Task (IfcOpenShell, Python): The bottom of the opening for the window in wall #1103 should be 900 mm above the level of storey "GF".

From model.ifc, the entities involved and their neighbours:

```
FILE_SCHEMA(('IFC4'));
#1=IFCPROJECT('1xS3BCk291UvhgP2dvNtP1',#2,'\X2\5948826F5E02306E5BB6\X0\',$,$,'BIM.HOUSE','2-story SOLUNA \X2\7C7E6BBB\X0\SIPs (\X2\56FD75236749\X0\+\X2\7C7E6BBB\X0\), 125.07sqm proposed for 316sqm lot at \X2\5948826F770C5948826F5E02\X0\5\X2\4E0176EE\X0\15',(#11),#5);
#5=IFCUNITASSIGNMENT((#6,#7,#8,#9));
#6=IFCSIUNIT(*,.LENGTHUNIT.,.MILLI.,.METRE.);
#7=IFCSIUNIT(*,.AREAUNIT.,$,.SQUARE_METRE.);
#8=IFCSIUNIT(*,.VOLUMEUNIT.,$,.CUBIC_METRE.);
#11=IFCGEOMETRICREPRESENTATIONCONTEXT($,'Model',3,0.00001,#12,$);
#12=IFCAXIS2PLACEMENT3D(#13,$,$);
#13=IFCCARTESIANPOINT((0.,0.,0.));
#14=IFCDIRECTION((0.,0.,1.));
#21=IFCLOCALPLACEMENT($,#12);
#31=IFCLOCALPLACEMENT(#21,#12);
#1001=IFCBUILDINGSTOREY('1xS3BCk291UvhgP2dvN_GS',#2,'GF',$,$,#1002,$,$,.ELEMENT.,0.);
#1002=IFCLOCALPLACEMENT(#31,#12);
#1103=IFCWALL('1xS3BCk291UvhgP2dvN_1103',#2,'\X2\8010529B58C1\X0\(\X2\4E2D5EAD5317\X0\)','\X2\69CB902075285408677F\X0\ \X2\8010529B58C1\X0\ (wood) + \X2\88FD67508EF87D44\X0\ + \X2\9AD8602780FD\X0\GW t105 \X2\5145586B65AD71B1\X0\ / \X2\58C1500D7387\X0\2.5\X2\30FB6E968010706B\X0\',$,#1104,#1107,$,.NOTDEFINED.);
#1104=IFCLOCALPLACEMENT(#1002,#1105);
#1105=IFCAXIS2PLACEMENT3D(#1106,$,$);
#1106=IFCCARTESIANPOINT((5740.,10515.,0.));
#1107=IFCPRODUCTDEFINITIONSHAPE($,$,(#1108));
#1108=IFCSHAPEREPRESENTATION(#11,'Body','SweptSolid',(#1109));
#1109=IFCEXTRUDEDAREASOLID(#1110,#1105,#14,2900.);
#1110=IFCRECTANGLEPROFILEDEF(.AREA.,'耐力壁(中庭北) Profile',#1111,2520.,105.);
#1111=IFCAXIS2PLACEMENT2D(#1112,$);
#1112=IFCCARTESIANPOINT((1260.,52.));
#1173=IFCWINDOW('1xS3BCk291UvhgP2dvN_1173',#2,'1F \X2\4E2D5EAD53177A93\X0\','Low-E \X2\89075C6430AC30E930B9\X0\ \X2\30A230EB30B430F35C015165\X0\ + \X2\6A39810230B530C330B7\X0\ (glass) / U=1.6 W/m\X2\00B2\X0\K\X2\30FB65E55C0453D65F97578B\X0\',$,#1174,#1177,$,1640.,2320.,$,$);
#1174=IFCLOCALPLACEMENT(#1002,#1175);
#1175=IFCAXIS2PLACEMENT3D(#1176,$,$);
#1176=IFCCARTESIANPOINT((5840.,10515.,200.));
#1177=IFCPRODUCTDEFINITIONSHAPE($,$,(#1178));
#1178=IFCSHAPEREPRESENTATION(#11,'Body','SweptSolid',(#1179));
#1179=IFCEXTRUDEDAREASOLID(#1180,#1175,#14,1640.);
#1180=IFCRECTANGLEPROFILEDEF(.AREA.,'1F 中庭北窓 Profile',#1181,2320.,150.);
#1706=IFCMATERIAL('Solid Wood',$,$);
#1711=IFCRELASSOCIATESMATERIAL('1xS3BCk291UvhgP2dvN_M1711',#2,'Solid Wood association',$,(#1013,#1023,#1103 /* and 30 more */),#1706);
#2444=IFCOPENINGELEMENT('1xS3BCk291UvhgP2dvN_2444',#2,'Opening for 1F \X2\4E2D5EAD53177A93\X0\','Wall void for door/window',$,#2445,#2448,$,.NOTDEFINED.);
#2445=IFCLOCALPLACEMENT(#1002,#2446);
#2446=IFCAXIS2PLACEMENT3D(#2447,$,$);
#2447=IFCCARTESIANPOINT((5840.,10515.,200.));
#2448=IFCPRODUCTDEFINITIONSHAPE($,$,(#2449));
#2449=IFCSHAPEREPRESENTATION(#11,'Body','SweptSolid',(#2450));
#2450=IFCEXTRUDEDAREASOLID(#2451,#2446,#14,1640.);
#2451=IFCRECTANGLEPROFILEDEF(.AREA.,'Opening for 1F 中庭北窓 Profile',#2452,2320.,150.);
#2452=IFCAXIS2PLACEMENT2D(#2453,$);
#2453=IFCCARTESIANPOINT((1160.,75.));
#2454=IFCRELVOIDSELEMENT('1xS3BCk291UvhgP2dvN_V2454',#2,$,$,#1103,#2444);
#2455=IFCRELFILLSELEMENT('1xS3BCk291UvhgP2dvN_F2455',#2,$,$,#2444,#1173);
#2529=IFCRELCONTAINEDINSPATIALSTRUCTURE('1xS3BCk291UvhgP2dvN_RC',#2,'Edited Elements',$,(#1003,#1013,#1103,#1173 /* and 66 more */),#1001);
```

```python
import numpy as np
import ifcopenshell
import ifcopenshell.api.geometry
import ifcopenshell.geom
import ifcopenshell.util.element
import ifcopenshell.util.placement
import ifcopenshell.util.shape
import ifcopenshell.util.unit

model = ifcopenshell.open("model.ifc")
unit_scale = ifcopenshell.util.unit.calculate_unit_scale(model)

window = model.by_guid("1xS3BCk291UvhgP2dvN_1173")
opening = window.FillsVoids[0].RelatingOpeningElement
storey = ifcopenshell.util.element.get_container(window, ifc_class="IfcBuildingStorey")
level = ifcopenshell.util.placement.get_local_placement(storey.ObjectPlacement)[2, 3]

# The opening's origin need not be at the sill, so measure its lowest point.
shape = ifcopenshell.geom.create_shape(ifcopenshell.geom.settings(), opening)
bottom = ifcopenshell.util.shape.get_shape_bottom_elevation(shape, shape.geometry) / unit_scale
dz = level + 0.9 / unit_scale - bottom

shift = np.array([0.0, 0.0, dz])
# The window is not placed relative to its opening, so move both.
for product in (opening, window):
    matrix = ifcopenshell.util.placement.get_local_placement(product.ObjectPlacement)
    matrix[:3, 3] += shift
    ifcopenshell.api.geometry.edit_object_placement(model, product=product, matrix=matrix, is_si=False)

print(f"moved by {dz * unit_scale:+.3f} m")

model.write("model_v2.ifc")
```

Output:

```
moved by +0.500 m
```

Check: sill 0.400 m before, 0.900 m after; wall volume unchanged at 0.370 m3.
